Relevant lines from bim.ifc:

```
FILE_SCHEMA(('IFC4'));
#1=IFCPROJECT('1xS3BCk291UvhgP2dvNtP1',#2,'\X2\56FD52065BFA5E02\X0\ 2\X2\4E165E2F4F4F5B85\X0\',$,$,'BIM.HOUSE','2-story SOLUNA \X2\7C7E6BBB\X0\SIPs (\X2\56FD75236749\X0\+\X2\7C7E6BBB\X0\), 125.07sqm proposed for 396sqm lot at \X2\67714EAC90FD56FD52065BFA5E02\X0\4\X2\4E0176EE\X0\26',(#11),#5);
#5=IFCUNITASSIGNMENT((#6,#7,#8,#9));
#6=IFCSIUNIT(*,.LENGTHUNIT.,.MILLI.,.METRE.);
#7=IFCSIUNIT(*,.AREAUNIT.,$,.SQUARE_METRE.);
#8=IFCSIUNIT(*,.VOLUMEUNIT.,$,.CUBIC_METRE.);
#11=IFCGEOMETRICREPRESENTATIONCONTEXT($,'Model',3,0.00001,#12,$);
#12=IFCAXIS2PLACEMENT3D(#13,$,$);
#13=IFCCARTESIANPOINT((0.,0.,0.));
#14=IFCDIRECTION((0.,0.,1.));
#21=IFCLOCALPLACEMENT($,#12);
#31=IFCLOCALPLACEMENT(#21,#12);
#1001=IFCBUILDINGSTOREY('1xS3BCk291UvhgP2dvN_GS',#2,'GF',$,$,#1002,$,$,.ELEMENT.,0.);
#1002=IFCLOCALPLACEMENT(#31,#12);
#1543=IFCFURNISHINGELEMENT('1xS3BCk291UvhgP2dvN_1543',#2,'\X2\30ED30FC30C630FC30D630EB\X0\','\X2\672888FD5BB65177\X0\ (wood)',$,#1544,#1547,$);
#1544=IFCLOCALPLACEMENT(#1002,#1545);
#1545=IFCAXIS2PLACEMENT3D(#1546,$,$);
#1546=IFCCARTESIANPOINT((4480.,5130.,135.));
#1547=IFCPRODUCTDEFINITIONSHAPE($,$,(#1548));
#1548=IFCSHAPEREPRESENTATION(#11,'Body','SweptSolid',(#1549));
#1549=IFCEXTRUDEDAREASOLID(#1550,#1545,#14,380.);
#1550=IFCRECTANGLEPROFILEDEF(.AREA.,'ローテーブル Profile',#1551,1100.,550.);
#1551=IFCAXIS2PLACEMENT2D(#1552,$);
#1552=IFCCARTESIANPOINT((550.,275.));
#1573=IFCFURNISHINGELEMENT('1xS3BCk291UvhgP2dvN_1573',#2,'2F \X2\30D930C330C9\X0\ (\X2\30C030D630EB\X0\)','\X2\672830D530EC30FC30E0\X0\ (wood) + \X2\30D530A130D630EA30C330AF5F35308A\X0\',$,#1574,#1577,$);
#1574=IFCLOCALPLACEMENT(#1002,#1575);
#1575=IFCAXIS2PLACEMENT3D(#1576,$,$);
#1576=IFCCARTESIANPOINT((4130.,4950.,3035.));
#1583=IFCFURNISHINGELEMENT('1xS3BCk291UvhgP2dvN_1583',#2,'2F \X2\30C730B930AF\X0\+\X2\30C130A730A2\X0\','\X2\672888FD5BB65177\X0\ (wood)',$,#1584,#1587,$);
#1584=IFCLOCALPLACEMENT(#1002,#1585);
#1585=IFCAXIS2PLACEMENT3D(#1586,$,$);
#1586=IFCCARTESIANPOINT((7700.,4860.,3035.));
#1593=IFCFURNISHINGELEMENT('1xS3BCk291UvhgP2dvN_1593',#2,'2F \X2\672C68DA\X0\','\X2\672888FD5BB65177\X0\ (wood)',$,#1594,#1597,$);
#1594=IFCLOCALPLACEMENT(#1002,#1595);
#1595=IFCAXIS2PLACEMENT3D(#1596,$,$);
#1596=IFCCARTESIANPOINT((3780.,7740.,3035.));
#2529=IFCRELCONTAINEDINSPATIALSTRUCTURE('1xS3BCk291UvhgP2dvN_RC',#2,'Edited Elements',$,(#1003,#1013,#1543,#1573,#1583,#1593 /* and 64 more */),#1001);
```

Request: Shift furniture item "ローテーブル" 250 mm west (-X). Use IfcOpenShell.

```python
import ifcopenshell
import ifcopenshell.api.geometry
import ifcopenshell.util.placement

model = ifcopenshell.open("bim.ifc")

item = model.by_guid("1xS3BCk291UvhgP2dvN_1543")
matrix = ifcopenshell.util.placement.get_local_placement(item.ObjectPlacement)
matrix[0, 3] -= 250.0
ifcopenshell.api.geometry.edit_object_placement(model, product=item, matrix=matrix, is_si=False)

print(ifcopenshell.util.placement.get_local_placement(item.ObjectPlacement).round(3) + 0.0)

model.write("bim_edited.ifc")
```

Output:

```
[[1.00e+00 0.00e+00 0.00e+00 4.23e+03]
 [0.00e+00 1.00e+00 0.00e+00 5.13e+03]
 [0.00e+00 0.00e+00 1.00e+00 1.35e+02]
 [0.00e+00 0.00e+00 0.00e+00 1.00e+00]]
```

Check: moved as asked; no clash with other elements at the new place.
